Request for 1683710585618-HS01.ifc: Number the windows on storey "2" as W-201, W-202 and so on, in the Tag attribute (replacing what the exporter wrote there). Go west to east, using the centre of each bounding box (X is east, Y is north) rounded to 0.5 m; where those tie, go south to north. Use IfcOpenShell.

First a look at what the model holds.

```python
import ifcopenshell
import ifcopenshell.util.element
import ifcopenshell.util.placement

model = ifcopenshell.open("1683710585618-HS01.ifc")
print(model.schema)
storey = next(s for s in model.by_type("IfcBuildingStorey") if s.Name == "2")
windows = [e for e in ifcopenshell.util.element.get_decomposition(storey) if e.is_a("IfcWindow")]
for e in sorted(windows, key=lambda e: e.id()):
    origin = ifcopenshell.util.placement.get_local_placement(e.ObjectPlacement)[:3, 3]
    print(e.id(), e.Tag, e.Name, origin.round(2) + 0.0, sep=" | ")
```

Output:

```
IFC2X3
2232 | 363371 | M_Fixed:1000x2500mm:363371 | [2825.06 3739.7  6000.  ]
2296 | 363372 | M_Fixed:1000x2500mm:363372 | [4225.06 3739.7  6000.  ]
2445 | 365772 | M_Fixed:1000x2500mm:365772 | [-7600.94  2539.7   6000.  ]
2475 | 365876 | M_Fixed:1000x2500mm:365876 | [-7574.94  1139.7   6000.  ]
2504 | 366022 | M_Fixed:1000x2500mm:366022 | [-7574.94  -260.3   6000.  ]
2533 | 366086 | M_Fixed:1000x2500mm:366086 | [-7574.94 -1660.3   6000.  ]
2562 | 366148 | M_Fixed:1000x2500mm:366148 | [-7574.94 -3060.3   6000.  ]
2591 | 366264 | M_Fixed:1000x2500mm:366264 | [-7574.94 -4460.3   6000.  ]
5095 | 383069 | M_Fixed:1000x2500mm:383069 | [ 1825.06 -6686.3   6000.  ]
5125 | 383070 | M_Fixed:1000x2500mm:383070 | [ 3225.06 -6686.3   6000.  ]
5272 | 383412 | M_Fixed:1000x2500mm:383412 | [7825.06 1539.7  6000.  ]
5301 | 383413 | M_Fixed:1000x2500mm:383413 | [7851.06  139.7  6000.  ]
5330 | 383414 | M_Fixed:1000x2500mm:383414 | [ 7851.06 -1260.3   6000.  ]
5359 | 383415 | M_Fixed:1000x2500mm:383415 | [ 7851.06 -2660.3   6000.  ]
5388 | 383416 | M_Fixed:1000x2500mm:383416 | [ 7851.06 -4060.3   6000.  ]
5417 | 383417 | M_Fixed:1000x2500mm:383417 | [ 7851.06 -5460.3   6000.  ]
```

```python
import ifcopenshell
import ifcopenshell.geom
import ifcopenshell.util.element
import ifcopenshell.util.shape

model = ifcopenshell.open("1683710585618-HS01.ifc")
settings = ifcopenshell.geom.settings()
settings.set("use-world-coords", True)


def centre(element):
    shape = ifcopenshell.geom.create_shape(settings, element)
    return ifcopenshell.util.shape.get_bbox_centroid(shape.geometry)


storey = next(s for s in model.by_type("IfcBuildingStorey") if s.Name == "2")
windows = [e for e in ifcopenshell.util.element.get_decomposition(storey) if e.is_a("IfcWindow")]

# Insertion points can sit at a corner or the storey origin, so sort by the geometry (in metres).
centres = {e: centre(e) for e in windows}
windows.sort(key=lambda e: (round(centres[e][0] / 0.5), centres[e][1]))

for i, e in enumerate(windows, start=1):
    number = f"W-2{i:02d}"
    e.Tag = number
    print(e.id(), number)

model.write("1683710585618-HS01_updated.ifc")
```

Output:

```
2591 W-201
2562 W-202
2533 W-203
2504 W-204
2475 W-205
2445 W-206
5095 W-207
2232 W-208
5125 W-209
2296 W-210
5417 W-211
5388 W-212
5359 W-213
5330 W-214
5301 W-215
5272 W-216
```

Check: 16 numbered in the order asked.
